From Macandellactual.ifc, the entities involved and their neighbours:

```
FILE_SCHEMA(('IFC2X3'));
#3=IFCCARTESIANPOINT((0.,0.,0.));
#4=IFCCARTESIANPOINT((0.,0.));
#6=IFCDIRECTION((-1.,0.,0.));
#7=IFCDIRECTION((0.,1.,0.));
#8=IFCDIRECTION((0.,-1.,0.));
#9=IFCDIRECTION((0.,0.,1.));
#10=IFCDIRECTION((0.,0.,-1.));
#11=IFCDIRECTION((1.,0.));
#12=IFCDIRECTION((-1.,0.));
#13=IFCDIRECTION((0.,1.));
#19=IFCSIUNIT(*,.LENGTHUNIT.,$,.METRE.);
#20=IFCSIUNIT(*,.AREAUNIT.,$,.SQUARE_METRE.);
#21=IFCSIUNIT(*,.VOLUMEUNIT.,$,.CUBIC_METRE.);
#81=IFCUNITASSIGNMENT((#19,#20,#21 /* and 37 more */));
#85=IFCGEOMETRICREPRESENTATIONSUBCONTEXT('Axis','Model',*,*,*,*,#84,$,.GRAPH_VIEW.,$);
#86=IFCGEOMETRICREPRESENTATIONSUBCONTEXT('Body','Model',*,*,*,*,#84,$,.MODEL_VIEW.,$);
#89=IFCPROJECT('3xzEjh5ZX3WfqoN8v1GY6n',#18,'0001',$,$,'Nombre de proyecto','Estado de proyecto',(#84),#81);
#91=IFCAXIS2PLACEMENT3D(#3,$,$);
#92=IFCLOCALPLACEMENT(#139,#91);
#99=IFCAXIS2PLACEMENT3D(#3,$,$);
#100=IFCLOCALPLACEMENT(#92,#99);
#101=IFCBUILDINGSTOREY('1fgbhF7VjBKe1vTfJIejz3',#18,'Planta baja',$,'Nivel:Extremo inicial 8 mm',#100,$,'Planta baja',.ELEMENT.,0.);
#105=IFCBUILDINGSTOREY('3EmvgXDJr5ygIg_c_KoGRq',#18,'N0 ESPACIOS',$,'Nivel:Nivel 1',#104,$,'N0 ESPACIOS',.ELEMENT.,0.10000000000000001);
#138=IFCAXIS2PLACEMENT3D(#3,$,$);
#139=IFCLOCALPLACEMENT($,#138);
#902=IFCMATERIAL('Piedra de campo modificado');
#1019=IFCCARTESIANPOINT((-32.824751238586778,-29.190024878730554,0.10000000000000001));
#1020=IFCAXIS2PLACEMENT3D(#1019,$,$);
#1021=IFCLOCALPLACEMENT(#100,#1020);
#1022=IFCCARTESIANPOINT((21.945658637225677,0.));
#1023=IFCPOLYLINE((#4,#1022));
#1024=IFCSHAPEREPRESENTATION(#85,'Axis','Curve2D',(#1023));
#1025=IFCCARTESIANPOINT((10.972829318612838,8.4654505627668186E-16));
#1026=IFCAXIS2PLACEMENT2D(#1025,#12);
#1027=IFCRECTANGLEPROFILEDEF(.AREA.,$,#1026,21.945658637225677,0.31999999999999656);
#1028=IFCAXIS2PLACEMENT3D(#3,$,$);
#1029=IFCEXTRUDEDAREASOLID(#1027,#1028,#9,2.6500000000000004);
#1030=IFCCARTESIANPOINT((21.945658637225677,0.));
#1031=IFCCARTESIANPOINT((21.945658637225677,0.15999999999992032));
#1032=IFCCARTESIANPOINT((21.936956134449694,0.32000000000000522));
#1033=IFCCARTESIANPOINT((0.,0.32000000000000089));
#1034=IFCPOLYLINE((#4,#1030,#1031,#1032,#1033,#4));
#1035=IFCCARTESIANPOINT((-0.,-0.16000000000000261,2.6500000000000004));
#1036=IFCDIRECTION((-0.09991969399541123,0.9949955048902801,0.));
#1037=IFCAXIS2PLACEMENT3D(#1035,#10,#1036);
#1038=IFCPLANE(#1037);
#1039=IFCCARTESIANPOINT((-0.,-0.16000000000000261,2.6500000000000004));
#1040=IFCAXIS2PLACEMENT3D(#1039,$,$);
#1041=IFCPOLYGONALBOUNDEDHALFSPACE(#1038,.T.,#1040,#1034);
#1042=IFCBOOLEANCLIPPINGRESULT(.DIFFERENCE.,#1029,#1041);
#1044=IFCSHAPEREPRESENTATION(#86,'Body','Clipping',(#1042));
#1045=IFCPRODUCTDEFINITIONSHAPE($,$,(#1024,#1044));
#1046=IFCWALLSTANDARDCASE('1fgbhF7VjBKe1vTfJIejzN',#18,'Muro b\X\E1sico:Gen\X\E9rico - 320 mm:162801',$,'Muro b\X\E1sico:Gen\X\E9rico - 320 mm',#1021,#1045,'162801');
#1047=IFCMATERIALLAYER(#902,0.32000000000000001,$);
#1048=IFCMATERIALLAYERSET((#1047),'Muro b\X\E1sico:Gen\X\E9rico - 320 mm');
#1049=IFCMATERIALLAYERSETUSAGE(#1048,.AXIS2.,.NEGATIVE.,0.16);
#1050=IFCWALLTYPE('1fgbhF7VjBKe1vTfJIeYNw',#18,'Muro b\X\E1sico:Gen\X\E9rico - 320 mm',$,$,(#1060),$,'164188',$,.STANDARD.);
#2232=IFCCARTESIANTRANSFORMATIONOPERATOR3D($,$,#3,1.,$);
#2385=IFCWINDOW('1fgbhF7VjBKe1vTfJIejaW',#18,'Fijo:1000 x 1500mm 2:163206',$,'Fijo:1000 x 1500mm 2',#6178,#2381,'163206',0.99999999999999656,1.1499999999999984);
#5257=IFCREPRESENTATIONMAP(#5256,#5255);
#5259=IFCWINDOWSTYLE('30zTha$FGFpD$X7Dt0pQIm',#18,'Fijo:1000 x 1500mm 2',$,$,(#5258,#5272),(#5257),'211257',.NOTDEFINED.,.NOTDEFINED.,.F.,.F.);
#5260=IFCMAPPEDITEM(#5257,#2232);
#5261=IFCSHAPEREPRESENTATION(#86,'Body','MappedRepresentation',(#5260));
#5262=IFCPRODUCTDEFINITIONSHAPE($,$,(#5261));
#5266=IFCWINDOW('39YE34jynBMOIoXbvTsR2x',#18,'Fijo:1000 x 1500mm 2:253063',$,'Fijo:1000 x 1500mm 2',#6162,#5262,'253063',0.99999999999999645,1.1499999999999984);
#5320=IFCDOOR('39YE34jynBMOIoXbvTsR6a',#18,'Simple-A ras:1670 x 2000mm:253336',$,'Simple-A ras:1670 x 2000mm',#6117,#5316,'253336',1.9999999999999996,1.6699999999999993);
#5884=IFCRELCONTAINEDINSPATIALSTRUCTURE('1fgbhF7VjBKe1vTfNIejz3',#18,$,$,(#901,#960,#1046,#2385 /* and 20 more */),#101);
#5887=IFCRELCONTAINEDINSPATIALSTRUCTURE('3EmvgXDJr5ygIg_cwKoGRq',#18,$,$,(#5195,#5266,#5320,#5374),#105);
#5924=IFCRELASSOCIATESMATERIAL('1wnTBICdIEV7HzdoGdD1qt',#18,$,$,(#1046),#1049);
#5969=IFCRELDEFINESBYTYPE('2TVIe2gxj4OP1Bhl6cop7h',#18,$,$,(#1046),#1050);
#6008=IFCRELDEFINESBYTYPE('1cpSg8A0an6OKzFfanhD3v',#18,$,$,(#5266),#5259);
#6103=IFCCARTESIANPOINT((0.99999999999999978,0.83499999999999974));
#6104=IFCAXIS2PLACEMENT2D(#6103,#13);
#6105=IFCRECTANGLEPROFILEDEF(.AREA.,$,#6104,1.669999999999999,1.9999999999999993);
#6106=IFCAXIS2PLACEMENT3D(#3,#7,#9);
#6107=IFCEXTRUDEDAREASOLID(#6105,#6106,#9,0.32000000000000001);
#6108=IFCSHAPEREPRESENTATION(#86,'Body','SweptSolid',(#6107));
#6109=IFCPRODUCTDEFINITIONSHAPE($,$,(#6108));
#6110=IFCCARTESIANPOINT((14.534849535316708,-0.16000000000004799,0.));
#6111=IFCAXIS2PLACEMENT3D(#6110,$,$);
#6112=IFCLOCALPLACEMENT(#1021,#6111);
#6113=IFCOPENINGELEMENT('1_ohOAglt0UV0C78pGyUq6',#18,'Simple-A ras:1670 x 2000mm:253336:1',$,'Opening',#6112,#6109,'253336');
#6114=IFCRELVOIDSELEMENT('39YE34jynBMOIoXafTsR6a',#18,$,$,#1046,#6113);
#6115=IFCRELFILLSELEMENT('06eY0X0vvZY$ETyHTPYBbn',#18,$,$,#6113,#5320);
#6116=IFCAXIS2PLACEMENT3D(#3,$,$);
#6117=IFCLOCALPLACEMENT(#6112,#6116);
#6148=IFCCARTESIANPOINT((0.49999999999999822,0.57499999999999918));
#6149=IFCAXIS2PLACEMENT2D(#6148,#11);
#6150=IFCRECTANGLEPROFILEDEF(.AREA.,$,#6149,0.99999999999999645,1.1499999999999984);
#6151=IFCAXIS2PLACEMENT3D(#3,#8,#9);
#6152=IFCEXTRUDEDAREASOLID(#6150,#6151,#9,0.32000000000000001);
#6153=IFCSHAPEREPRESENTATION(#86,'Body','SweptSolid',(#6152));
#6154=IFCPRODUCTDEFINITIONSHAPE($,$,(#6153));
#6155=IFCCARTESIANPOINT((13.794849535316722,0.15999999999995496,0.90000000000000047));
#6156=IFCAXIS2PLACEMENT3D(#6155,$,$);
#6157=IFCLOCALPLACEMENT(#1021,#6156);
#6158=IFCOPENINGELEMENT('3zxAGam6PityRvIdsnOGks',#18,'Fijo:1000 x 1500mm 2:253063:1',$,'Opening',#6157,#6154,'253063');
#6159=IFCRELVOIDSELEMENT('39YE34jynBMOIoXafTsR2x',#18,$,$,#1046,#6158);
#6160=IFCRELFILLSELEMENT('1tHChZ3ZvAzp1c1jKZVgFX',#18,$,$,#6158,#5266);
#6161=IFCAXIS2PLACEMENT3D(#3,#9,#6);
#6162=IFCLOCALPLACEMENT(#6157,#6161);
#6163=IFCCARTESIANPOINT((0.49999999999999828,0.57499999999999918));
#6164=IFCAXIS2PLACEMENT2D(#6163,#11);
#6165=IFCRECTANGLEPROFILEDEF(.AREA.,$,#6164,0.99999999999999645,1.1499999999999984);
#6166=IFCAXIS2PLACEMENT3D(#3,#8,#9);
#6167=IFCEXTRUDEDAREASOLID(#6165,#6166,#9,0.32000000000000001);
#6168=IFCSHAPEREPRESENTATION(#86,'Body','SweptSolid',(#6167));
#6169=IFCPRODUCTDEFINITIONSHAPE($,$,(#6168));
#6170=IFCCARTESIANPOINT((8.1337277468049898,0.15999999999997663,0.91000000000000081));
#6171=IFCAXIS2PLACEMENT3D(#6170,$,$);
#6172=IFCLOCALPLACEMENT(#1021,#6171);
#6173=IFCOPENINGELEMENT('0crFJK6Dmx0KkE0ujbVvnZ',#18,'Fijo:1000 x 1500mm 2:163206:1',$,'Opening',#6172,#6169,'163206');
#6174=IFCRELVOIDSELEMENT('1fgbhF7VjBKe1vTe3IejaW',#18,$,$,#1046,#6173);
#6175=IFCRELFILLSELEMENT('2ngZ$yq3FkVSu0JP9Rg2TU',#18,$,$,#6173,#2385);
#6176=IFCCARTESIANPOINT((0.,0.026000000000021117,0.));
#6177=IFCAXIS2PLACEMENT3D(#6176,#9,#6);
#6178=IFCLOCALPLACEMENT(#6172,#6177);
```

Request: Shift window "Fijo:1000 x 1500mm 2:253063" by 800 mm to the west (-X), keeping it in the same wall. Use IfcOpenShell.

```python
import ifcopenshell
import ifcopenshell.api.geometry
import ifcopenshell.util.placement

model = ifcopenshell.open("Macandellactual.ifc")

window = model.by_guid("39YE34jynBMOIoXbvTsR2x")
opening = window.FillsVoids[0].RelatingOpeningElement
wall = opening.VoidsElements[0].RelatingBuildingElement

wall_matrix = ifcopenshell.util.placement.get_local_placement(wall.ObjectPlacement)
shift = wall_matrix[:3, 0] * -0.8
before = ifcopenshell.util.placement.get_local_placement(window.ObjectPlacement)[:3, 3].copy()

# The window is placed relative to its opening, so it follows when the opening moves.
matrix = ifcopenshell.util.placement.get_local_placement(opening.ObjectPlacement)
matrix[:3, 3] += shift
ifcopenshell.api.geometry.edit_object_placement(
    model, product=opening, matrix=matrix, is_si=False, should_transform_children=True
)

after = ifcopenshell.util.placement.get_local_placement(window.ObjectPlacement)[:3, 3]
print("window moved by", (after - before).round(3) + 0.0)

model.write("Macandellactual_rev.ifc")
```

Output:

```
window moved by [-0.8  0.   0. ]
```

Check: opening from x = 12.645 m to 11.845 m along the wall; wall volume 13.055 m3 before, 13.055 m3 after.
